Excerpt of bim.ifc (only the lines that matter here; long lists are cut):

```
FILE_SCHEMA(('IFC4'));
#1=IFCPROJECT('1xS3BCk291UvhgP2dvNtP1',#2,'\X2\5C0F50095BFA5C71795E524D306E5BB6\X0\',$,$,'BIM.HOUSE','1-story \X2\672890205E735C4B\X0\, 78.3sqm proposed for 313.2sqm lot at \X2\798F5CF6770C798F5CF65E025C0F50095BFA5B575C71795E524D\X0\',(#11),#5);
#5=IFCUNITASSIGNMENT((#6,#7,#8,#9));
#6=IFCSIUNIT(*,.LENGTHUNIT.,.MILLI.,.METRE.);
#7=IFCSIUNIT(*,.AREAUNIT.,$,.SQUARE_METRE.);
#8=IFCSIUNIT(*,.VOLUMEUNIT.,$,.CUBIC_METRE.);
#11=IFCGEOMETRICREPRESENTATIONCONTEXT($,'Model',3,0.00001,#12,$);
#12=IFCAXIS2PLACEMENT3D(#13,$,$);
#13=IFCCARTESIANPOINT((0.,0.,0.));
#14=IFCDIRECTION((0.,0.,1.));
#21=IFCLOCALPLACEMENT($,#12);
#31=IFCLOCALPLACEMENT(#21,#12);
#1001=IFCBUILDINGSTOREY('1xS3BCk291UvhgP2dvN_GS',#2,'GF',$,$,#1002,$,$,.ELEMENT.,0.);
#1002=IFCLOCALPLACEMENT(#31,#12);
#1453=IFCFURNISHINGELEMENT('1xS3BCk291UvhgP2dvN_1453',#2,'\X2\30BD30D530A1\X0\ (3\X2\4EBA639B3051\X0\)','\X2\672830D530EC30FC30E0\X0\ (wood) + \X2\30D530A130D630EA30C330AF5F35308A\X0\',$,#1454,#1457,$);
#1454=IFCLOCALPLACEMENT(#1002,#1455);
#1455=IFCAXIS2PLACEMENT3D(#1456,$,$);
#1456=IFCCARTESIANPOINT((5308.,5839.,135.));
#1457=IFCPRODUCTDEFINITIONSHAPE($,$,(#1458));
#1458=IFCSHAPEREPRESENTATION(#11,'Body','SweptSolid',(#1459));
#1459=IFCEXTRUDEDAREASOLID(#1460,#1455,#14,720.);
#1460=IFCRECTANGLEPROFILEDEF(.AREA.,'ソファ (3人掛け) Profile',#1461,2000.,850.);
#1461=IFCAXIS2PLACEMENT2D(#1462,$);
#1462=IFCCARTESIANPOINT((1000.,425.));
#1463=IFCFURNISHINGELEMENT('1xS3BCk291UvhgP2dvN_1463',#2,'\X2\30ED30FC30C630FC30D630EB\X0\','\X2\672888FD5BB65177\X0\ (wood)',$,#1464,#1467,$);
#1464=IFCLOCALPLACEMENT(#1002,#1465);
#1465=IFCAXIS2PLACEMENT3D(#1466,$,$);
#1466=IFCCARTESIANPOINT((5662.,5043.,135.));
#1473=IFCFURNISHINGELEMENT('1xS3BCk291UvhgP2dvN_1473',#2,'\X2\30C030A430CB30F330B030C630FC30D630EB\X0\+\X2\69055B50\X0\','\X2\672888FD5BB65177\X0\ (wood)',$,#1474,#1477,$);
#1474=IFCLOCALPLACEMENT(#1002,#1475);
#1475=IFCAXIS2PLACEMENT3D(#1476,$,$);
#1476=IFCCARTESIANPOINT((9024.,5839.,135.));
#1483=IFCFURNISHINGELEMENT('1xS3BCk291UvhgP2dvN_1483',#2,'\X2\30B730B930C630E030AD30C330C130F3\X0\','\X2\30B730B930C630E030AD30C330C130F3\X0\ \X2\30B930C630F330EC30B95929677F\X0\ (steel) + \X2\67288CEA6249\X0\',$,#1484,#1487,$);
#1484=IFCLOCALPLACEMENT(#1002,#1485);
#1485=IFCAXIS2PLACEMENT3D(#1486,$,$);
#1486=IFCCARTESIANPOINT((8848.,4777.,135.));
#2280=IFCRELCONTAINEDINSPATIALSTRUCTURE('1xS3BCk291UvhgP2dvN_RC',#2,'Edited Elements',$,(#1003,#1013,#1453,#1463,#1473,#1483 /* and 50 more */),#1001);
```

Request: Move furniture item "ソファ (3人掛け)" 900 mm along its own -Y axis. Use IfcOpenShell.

```python
import ifcopenshell
import ifcopenshell.api.geometry
import ifcopenshell.util.placement

model = ifcopenshell.open("bim.ifc")

item = model.by_guid("1xS3BCk291UvhgP2dvN_1453")
matrix = ifcopenshell.util.placement.get_local_placement(item.ObjectPlacement)
matrix[:3, 3] -= matrix[:3, 1] * 900.0
ifcopenshell.api.geometry.edit_object_placement(model, product=item, matrix=matrix, is_si=False)

print(ifcopenshell.util.placement.get_local_placement(item.ObjectPlacement).round(3) + 0.0)

model.write("bim_rev.ifc")
```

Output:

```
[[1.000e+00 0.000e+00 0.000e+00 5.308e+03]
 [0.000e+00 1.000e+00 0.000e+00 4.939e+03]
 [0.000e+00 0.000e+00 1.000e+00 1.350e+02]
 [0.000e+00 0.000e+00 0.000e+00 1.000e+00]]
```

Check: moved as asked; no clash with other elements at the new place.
